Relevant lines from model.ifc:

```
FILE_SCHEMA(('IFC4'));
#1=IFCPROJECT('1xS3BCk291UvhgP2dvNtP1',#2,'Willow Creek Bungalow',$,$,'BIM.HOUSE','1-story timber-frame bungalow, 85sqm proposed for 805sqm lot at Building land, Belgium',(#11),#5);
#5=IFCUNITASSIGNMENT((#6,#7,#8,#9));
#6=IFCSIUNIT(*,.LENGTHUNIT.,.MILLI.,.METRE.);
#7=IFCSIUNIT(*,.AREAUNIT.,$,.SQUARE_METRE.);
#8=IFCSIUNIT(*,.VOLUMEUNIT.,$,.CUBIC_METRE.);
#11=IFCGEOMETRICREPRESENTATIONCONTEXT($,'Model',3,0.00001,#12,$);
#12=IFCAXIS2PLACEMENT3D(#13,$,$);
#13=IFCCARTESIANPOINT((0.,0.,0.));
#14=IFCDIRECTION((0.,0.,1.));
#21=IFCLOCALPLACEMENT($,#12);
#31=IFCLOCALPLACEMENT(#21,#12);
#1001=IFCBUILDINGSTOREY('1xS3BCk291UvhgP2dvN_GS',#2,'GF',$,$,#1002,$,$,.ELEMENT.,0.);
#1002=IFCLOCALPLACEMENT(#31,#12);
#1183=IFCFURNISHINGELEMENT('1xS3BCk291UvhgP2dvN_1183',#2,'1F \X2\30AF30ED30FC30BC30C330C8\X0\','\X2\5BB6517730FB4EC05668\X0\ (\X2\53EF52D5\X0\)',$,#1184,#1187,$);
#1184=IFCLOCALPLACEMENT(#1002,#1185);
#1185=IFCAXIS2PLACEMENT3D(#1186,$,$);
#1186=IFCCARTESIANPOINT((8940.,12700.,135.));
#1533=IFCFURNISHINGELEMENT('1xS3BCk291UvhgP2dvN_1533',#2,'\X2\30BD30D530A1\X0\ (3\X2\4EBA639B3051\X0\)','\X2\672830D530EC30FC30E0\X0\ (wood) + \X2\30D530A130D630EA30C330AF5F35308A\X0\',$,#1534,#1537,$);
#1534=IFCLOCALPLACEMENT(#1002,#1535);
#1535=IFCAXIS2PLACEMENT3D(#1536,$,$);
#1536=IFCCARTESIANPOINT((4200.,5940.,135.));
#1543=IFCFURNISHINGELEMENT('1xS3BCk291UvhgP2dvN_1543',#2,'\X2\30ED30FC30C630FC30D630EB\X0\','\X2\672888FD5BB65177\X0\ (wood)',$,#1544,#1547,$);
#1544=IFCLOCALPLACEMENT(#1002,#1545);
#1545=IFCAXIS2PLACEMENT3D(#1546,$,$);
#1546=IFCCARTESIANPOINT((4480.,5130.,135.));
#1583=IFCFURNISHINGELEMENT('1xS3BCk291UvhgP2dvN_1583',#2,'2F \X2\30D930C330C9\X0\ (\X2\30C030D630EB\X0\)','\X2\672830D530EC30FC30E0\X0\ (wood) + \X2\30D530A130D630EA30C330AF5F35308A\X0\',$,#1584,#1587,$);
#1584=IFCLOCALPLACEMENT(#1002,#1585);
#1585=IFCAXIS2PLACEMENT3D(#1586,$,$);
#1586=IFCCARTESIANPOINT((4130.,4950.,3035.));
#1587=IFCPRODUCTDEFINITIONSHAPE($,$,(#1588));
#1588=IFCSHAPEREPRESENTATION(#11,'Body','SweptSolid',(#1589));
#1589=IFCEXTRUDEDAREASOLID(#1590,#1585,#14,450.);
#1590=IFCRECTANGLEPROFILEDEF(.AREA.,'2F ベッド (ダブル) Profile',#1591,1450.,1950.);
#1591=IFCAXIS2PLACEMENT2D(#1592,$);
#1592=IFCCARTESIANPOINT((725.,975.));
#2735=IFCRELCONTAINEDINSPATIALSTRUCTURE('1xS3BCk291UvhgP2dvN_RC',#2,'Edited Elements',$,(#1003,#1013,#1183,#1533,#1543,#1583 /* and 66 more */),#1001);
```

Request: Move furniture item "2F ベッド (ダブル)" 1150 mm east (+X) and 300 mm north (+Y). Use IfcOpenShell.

```python
import ifcopenshell
import ifcopenshell.api.geometry
import ifcopenshell.util.placement
import ifcopenshell.util.unit

model = ifcopenshell.open("model.ifc")
unit_scale = ifcopenshell.util.unit.calculate_unit_scale(model)

item = model.by_guid("1xS3BCk291UvhgP2dvN_1583")
matrix = ifcopenshell.util.placement.get_local_placement(item.ObjectPlacement)
matrix[0, 3] += 1.15 / unit_scale
matrix[1, 3] += 0.3 / unit_scale
ifcopenshell.api.geometry.edit_object_placement(model, product=item, matrix=matrix, is_si=False)

print(ifcopenshell.util.placement.get_local_placement(item.ObjectPlacement).round(3) + 0.0)

model.write("model_rev.ifc")
```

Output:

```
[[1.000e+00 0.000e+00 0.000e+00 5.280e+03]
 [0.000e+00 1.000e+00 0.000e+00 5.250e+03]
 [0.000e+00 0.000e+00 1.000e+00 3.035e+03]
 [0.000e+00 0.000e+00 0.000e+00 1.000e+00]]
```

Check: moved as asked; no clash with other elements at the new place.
